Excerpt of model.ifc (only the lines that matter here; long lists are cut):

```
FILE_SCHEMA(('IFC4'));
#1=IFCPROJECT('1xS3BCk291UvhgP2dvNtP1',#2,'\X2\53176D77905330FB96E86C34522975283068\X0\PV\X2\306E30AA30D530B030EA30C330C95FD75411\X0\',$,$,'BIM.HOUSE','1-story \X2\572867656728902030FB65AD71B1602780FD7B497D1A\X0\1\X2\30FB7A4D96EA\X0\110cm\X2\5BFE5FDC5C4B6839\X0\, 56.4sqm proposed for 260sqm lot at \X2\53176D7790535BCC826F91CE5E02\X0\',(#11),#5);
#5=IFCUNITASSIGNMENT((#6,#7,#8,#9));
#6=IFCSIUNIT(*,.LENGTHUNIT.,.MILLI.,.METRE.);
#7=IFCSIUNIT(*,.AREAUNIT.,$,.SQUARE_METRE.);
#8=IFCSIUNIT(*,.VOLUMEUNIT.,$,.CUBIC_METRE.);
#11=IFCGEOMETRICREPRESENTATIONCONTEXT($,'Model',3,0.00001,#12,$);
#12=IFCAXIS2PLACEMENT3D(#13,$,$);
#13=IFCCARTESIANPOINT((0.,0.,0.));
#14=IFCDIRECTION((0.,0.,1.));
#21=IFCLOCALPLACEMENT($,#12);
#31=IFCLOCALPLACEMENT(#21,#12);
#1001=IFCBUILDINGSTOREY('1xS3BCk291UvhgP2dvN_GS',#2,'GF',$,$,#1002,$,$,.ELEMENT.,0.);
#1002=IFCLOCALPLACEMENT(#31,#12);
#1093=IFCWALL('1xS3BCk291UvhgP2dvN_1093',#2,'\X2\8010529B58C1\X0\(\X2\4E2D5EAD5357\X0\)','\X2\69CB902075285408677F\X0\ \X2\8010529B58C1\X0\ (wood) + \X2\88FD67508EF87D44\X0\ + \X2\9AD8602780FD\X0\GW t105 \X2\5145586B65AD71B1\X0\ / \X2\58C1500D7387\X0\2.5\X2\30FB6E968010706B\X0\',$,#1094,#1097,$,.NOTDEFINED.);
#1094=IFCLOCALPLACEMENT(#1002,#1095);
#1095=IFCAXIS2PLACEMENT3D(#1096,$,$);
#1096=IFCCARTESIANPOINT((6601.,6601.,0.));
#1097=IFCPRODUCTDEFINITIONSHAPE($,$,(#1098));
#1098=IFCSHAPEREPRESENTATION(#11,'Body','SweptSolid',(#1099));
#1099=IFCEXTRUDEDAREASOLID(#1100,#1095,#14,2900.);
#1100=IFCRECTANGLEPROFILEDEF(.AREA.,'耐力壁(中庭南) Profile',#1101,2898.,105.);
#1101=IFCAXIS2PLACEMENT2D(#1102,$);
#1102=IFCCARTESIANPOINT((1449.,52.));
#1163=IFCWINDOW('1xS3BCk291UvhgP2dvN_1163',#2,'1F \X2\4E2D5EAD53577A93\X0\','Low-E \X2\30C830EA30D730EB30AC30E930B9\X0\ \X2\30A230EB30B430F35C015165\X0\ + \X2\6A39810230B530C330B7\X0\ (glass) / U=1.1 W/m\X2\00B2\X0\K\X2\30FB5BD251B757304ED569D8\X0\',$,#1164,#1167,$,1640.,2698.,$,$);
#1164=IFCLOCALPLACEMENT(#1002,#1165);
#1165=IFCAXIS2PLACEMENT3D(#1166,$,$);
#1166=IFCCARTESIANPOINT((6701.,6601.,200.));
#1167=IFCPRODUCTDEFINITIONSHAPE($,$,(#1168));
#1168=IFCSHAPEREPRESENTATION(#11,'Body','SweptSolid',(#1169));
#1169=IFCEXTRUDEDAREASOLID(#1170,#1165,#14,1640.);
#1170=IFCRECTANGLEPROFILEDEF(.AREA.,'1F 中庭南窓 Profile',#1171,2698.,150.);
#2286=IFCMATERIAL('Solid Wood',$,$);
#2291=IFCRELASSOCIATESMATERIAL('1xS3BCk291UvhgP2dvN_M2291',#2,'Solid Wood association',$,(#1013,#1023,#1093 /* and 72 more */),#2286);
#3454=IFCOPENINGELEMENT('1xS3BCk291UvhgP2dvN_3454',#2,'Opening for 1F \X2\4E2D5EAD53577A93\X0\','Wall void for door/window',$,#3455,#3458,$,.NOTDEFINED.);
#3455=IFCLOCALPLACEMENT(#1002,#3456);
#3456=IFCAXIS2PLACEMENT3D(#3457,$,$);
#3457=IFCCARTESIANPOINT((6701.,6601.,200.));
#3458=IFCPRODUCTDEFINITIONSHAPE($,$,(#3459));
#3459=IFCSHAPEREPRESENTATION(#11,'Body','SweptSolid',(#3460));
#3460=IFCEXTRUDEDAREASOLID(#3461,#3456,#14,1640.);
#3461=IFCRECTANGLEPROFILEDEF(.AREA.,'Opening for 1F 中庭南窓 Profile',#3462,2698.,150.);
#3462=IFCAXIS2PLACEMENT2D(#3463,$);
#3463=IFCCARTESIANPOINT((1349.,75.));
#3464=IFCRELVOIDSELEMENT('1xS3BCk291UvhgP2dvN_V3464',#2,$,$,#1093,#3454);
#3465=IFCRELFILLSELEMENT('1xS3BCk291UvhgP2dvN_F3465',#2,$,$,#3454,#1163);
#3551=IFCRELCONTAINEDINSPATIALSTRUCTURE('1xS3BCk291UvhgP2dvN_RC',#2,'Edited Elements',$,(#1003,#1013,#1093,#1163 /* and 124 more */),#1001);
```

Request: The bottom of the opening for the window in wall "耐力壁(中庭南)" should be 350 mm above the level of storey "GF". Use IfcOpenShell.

```python
import numpy as np
import ifcopenshell
import ifcopenshell.api.geometry
import ifcopenshell.geom
import ifcopenshell.util.element
import ifcopenshell.util.placement
import ifcopenshell.util.shape
import ifcopenshell.util.unit

model = ifcopenshell.open("model.ifc")
unit_scale = ifcopenshell.util.unit.calculate_unit_scale(model)

window = model.by_guid("1xS3BCk291UvhgP2dvN_1163")
opening = window.FillsVoids[0].RelatingOpeningElement
storey = ifcopenshell.util.element.get_container(window, ifc_class="IfcBuildingStorey")
level = ifcopenshell.util.placement.get_local_placement(storey.ObjectPlacement)[2, 3]

# The opening's origin need not be at the sill, so measure its lowest point.
shape = ifcopenshell.geom.create_shape(ifcopenshell.geom.settings(), opening)
bottom = ifcopenshell.util.shape.get_shape_bottom_elevation(shape, shape.geometry) / unit_scale
dz = level + 350.0 - bottom

shift = np.array([0.0, 0.0, dz])
# The window is not placed relative to its opening, so move both.
for product in (opening, window):
    matrix = ifcopenshell.util.placement.get_local_placement(product.ObjectPlacement)
    matrix[:3, 3] += shift
    ifcopenshell.api.geometry.edit_object_placement(model, product=product, matrix=matrix, is_si=False)

print(f"moved by {dz * unit_scale:+.3f} m")

model.write("model_rev.ifc")
```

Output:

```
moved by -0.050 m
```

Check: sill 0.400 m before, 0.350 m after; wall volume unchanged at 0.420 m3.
